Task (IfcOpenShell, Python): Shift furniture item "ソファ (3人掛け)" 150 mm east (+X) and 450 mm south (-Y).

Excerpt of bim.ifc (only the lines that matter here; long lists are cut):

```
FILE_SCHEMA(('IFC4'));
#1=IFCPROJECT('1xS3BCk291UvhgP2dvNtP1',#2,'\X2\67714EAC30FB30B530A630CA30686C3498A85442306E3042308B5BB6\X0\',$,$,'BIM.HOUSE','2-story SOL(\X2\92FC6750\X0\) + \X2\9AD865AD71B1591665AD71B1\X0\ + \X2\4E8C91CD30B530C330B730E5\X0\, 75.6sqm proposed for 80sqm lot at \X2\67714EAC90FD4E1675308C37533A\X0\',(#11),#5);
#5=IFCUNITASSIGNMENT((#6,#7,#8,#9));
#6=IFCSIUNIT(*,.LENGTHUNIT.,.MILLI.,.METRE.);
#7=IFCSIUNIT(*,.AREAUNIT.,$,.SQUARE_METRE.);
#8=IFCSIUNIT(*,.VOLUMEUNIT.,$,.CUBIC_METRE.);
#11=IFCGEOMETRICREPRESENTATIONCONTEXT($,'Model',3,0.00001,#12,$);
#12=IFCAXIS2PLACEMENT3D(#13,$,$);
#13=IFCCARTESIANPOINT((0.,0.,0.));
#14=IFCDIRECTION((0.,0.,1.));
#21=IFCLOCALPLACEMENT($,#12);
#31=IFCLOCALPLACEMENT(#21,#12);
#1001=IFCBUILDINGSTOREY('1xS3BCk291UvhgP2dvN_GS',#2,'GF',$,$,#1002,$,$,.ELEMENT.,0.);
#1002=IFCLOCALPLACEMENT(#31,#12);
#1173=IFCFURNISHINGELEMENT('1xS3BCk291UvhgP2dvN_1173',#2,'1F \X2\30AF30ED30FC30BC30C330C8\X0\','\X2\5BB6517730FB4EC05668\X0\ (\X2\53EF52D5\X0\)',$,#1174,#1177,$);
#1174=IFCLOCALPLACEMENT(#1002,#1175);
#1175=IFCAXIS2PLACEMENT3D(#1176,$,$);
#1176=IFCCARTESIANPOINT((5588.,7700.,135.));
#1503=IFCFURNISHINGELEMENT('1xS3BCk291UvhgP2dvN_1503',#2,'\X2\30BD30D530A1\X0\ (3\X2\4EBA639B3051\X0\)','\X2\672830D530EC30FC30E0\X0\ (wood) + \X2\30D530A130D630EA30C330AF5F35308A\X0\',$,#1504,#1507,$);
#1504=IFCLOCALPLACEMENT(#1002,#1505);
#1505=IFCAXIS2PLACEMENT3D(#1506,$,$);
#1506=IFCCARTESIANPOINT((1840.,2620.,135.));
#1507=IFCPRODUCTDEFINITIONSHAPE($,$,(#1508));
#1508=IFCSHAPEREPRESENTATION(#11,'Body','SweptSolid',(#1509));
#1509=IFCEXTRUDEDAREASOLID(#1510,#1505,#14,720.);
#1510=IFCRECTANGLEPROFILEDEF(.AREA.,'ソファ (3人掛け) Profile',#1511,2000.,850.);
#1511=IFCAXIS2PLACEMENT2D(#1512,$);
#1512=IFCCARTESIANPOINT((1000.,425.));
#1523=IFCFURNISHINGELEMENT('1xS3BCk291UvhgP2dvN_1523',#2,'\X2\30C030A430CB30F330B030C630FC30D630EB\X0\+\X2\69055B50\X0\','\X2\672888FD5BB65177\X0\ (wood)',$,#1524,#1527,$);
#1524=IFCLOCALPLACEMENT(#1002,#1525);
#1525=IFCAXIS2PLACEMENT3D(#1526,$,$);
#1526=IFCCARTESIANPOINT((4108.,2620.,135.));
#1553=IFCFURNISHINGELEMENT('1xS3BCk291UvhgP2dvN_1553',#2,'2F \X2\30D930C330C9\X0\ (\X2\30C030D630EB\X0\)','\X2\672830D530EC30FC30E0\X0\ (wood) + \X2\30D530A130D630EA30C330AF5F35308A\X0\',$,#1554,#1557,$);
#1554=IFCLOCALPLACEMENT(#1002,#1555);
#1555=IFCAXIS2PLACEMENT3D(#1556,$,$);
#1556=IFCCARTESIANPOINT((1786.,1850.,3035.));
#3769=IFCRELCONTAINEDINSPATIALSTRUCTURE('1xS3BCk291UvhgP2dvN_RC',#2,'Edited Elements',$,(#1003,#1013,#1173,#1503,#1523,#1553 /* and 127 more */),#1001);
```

```python
import ifcopenshell
import ifcopenshell.api.geometry
import ifcopenshell.util.placement

model = ifcopenshell.open("bim.ifc")

item = model.by_guid("1xS3BCk291UvhgP2dvN_1503")
matrix = ifcopenshell.util.placement.get_local_placement(item.ObjectPlacement)
matrix[0, 3] += 150.0
matrix[1, 3] -= 450.0
ifcopenshell.api.geometry.edit_object_placement(model, product=item, matrix=matrix, is_si=False)

print(ifcopenshell.util.placement.get_local_placement(item.ObjectPlacement).round(3) + 0.0)

model.write("bim_rev.ifc")
```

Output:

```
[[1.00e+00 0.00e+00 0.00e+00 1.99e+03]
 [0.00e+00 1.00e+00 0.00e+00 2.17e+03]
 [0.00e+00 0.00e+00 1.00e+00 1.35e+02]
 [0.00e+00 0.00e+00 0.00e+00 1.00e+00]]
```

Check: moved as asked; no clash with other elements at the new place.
